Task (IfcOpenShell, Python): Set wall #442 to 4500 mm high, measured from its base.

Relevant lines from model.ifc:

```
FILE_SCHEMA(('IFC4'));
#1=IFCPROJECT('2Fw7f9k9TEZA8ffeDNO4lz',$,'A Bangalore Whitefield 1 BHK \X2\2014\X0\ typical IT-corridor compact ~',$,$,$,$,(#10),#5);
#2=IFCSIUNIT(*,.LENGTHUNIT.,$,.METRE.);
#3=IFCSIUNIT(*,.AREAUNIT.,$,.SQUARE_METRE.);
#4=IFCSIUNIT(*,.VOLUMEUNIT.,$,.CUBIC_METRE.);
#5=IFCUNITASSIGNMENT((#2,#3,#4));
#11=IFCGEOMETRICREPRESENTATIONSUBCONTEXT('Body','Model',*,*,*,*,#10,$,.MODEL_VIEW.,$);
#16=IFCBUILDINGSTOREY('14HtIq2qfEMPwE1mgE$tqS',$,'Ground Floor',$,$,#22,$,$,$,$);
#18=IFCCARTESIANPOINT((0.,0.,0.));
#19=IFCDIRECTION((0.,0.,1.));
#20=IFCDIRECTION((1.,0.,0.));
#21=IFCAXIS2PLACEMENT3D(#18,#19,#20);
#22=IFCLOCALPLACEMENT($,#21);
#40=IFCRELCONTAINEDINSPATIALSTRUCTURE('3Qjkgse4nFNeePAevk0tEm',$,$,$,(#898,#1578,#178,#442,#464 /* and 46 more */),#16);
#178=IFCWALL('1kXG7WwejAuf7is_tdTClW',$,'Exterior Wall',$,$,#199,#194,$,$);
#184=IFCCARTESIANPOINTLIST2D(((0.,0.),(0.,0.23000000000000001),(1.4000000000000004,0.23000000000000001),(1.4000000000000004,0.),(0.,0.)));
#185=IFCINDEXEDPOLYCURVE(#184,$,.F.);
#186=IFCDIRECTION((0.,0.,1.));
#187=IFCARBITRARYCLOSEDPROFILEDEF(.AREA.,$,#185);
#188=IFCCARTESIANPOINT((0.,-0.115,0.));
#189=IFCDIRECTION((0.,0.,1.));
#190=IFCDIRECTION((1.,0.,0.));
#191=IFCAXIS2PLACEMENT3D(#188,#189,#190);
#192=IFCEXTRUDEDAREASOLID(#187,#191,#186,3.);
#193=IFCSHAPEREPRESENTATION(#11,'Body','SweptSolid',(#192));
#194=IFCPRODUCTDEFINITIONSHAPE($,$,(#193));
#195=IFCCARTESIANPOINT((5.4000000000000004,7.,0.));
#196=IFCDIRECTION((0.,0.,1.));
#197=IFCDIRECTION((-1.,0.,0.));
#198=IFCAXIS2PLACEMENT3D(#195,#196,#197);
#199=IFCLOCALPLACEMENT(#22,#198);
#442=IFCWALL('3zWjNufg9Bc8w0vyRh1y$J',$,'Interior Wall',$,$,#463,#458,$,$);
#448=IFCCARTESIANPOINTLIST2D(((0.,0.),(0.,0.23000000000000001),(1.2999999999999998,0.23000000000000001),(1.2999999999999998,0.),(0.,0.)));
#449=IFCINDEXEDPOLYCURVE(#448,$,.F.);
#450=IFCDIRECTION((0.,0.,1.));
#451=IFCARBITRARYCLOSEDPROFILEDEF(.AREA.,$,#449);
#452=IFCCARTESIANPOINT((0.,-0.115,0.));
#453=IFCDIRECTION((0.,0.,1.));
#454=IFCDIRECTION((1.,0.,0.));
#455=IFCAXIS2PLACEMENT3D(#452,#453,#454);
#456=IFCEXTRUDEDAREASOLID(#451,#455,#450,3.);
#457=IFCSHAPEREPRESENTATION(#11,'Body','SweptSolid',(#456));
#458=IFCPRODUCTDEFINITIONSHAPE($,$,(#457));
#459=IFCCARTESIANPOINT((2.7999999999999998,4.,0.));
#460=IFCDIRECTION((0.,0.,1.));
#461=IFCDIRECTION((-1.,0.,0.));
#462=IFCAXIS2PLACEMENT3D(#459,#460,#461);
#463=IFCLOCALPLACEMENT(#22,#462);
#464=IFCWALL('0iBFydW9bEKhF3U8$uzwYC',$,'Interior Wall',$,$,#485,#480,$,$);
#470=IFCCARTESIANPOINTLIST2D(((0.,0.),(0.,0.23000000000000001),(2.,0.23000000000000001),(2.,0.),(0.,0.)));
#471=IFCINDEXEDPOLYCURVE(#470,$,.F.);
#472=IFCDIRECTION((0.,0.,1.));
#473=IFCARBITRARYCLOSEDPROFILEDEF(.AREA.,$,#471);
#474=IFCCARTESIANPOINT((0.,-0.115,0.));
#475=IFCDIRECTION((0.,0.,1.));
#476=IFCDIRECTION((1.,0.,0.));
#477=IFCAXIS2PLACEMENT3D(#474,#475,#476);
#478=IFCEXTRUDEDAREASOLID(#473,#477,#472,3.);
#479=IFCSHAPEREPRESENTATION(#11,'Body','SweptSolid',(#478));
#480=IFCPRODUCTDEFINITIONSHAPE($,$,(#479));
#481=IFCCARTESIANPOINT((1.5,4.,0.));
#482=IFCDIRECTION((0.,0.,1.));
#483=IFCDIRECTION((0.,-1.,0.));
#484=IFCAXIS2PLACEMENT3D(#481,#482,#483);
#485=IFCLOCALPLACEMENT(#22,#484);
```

```python
import ifcopenshell
import ifcopenshell.geom
import ifcopenshell.util.representation
import ifcopenshell.util.shape
import ifcopenshell.util.unit

model = ifcopenshell.open("model.ifc")
unit_scale = ifcopenshell.util.unit.calculate_unit_scale(model)
settings = ifcopenshell.geom.settings()


def volume(element):
    """Net volume in cubic metres, openings subtracted."""
    shape = ifcopenshell.geom.create_shape(settings, element)
    return ifcopenshell.util.shape.get_volume(shape.geometry)


wall = model.by_guid("3zWjNufg9Bc8w0vyRh1y$J")
before = volume(wall)

body = ifcopenshell.util.representation.get_representation(wall, "Model", "Body")
solid = body.Items[0]
old_height = solid.Depth
solid.Depth = 4.5 / unit_scale
after = volume(wall)

print(f"height {old_height:g} -> {solid.Depth:g}, volume {before:.3f} -> {after:.3f} m3")

model.write("model_v2.ifc")
```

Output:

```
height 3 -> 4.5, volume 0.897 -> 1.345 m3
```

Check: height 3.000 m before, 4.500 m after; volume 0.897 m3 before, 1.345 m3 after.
